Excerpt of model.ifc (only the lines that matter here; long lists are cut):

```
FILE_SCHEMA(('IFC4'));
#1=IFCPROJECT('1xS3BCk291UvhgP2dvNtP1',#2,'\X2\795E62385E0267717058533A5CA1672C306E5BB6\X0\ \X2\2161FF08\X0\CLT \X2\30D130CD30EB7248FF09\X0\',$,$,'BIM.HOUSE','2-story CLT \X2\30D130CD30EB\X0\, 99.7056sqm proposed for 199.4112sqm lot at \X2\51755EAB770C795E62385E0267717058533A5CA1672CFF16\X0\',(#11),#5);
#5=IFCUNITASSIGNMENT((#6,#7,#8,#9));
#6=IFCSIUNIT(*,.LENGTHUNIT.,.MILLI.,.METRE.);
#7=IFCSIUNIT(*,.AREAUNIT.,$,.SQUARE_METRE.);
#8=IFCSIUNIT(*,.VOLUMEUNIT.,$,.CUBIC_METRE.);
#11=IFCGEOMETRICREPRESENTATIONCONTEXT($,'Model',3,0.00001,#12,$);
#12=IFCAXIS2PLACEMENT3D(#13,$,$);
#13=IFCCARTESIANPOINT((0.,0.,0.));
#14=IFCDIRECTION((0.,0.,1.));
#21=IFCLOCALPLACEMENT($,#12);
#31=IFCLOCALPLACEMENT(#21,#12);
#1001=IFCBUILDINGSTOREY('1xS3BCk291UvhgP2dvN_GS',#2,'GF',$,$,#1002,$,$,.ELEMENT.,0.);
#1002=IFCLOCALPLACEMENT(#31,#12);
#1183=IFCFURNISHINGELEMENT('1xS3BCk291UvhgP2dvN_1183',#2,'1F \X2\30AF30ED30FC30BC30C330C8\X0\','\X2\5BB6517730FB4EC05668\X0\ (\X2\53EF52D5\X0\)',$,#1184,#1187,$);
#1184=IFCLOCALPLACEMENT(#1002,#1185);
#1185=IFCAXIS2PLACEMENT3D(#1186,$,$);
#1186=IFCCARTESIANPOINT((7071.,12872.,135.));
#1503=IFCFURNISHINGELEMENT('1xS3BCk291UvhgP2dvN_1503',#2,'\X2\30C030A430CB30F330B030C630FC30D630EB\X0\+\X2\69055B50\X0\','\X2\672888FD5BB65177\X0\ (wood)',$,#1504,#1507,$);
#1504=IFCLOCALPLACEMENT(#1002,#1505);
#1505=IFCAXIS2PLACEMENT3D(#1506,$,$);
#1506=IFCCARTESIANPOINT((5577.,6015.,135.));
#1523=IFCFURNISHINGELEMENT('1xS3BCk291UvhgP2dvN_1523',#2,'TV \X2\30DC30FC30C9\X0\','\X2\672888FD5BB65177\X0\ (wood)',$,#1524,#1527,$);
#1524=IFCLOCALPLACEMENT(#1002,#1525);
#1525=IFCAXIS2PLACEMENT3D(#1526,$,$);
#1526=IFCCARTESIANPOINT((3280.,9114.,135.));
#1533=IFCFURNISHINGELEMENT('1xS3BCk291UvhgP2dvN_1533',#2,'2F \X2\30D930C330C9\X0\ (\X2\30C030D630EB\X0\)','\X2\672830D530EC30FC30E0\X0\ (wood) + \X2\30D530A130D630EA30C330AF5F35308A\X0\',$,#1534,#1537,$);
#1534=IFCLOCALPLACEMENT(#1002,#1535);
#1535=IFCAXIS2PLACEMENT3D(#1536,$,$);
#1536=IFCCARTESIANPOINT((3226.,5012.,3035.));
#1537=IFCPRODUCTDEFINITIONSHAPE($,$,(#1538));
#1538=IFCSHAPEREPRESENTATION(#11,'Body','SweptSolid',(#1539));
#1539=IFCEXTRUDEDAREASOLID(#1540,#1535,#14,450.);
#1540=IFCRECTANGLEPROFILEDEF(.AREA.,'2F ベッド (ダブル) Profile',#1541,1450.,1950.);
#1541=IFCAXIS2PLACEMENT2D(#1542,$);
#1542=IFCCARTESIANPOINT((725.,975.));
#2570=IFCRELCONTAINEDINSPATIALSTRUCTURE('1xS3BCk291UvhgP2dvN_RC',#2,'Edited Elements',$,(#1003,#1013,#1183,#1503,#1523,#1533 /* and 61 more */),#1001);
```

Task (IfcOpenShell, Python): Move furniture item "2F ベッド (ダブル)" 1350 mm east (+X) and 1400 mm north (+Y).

```python
import ifcopenshell
import ifcopenshell.api.geometry
import ifcopenshell.util.placement

model = ifcopenshell.open("model.ifc")

item = model.by_guid("1xS3BCk291UvhgP2dvN_1533")
matrix = ifcopenshell.util.placement.get_local_placement(item.ObjectPlacement)
matrix[0, 3] += 1350.0
matrix[1, 3] += 1400.0
ifcopenshell.api.geometry.edit_object_placement(model, product=item, matrix=matrix, is_si=False)

print(ifcopenshell.util.placement.get_local_placement(item.ObjectPlacement).round(3) + 0.0)

model.write("model_updated.ifc")
```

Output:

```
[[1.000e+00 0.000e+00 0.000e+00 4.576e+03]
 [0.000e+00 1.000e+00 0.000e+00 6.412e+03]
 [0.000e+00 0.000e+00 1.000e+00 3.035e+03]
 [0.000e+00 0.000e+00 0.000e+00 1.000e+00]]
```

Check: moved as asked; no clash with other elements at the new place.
